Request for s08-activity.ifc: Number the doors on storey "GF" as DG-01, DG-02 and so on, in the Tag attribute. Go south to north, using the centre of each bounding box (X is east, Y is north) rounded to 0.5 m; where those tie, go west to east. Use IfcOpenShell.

First a look at what the model holds.

```python
import ifcopenshell
import ifcopenshell.util.element
import ifcopenshell.util.placement

model = ifcopenshell.open("s08-activity.ifc")
print(model.schema)
storey = next(s for s in model.by_type("IfcBuildingStorey") if s.Name == "GF")
doors = [e for e in ifcopenshell.util.element.get_decomposition(storey) if e.is_a("IfcDoor")]
for e in sorted(doors, key=lambda e: e.id()):
    origin = ifcopenshell.util.placement.get_local_placement(e.ObjectPlacement)[:3, 3]
    print(e.id(), e.Tag, e.Name, origin.round(2) + 0.0, sep=" | ")
```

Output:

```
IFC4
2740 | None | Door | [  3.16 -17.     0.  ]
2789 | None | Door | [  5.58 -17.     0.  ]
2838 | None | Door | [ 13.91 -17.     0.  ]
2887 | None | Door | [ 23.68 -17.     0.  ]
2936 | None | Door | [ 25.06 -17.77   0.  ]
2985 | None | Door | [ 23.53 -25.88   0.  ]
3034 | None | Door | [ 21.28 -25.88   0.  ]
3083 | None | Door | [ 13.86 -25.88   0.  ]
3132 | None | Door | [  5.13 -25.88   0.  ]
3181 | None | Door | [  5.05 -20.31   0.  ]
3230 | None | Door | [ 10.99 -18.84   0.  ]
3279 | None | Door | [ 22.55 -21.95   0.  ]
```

```python
import ifcopenshell
import ifcopenshell.geom
import ifcopenshell.util.element
import ifcopenshell.util.shape

model = ifcopenshell.open("s08-activity.ifc")
settings = ifcopenshell.geom.settings()
settings.set("use-world-coords", True)


def centre(element):
    shape = ifcopenshell.geom.create_shape(settings, element)
    return ifcopenshell.util.shape.get_bbox_centroid(shape.geometry)


storey = next(s for s in model.by_type("IfcBuildingStorey") if s.Name == "GF")
doors = [e for e in ifcopenshell.util.element.get_decomposition(storey) if e.is_a("IfcDoor")]

# Insertion points can sit at a corner or the storey origin, so sort by the geometry (in metres).
centres = {e: centre(e) for e in doors}
doors.sort(key=lambda e: (round(centres[e][1] / 0.5), centres[e][0]))

for i, e in enumerate(doors, start=1):
    number = f"DG-{i:02d}"
    e.Tag = number
    print(e.id(), number)

model.write("s08-activity_updated.ifc")
```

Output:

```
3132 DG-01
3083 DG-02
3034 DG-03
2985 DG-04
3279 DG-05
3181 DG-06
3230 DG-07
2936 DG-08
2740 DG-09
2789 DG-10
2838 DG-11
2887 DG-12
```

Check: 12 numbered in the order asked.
